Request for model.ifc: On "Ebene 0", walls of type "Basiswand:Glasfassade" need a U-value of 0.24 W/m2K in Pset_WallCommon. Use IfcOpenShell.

First a look at what the model holds.

```python
import ifcopenshell
import ifcopenshell.util.element

model = ifcopenshell.open("model.ifc")
print(model.schema)
storey = next(s for s in model.by_type("IfcBuildingStorey") if s.Name == "Ebene 0")
walls = [e for e in ifcopenshell.util.element.get_decomposition(storey) if e.is_a("IfcWall")]
seen = {}
for e in walls:
    element_type = ifcopenshell.util.element.get_type(e)
    key = (element_type.Name if element_type != e and element_type else None, ifcopenshell.util.element.get_pset(e, "Pset_WallCommon", "ThermalTransmittance"))
    seen[key] = seen.get(key, 0) + 1
for (name, value), count in sorted(seen.items(), key=str):
    print(count, "x", name, "|", value)
```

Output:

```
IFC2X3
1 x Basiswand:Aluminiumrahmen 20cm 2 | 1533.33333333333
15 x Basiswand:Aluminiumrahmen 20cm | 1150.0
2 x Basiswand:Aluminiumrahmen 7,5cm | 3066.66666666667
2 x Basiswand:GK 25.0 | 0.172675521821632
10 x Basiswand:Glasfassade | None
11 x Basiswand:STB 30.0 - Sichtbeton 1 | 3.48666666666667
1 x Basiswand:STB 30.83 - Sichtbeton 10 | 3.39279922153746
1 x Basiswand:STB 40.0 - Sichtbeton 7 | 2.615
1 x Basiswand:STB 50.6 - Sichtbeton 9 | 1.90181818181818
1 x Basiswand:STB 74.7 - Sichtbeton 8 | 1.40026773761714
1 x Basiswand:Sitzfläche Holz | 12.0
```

```python
import ifcopenshell
import ifcopenshell.api.pset
import ifcopenshell.util.element

model = ifcopenshell.open("model.ifc")

storey = next(s for s in model.by_type("IfcBuildingStorey") if s.Name == "Ebene 0")
walls = [e for e in ifcopenshell.util.element.get_decomposition(storey) if e.is_a("IfcWall")]

count = 0
for e in walls:
    element_type = ifcopenshell.util.element.get_type(e)
    if element_type in (None, e) or element_type.Name != "Basiswand:Glasfassade":
        continue
    # add_pset returns the element's existing set when there is one.
    pset = ifcopenshell.api.pset.add_pset(model, product=e, name="Pset_WallCommon")
    ifcopenshell.api.pset.edit_pset(model, pset=pset, properties={"ThermalTransmittance": 0.24})
    count += 1

print(count, "walls updated")

model.write("model_v2.ifc")
```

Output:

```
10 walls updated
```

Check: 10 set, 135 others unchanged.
